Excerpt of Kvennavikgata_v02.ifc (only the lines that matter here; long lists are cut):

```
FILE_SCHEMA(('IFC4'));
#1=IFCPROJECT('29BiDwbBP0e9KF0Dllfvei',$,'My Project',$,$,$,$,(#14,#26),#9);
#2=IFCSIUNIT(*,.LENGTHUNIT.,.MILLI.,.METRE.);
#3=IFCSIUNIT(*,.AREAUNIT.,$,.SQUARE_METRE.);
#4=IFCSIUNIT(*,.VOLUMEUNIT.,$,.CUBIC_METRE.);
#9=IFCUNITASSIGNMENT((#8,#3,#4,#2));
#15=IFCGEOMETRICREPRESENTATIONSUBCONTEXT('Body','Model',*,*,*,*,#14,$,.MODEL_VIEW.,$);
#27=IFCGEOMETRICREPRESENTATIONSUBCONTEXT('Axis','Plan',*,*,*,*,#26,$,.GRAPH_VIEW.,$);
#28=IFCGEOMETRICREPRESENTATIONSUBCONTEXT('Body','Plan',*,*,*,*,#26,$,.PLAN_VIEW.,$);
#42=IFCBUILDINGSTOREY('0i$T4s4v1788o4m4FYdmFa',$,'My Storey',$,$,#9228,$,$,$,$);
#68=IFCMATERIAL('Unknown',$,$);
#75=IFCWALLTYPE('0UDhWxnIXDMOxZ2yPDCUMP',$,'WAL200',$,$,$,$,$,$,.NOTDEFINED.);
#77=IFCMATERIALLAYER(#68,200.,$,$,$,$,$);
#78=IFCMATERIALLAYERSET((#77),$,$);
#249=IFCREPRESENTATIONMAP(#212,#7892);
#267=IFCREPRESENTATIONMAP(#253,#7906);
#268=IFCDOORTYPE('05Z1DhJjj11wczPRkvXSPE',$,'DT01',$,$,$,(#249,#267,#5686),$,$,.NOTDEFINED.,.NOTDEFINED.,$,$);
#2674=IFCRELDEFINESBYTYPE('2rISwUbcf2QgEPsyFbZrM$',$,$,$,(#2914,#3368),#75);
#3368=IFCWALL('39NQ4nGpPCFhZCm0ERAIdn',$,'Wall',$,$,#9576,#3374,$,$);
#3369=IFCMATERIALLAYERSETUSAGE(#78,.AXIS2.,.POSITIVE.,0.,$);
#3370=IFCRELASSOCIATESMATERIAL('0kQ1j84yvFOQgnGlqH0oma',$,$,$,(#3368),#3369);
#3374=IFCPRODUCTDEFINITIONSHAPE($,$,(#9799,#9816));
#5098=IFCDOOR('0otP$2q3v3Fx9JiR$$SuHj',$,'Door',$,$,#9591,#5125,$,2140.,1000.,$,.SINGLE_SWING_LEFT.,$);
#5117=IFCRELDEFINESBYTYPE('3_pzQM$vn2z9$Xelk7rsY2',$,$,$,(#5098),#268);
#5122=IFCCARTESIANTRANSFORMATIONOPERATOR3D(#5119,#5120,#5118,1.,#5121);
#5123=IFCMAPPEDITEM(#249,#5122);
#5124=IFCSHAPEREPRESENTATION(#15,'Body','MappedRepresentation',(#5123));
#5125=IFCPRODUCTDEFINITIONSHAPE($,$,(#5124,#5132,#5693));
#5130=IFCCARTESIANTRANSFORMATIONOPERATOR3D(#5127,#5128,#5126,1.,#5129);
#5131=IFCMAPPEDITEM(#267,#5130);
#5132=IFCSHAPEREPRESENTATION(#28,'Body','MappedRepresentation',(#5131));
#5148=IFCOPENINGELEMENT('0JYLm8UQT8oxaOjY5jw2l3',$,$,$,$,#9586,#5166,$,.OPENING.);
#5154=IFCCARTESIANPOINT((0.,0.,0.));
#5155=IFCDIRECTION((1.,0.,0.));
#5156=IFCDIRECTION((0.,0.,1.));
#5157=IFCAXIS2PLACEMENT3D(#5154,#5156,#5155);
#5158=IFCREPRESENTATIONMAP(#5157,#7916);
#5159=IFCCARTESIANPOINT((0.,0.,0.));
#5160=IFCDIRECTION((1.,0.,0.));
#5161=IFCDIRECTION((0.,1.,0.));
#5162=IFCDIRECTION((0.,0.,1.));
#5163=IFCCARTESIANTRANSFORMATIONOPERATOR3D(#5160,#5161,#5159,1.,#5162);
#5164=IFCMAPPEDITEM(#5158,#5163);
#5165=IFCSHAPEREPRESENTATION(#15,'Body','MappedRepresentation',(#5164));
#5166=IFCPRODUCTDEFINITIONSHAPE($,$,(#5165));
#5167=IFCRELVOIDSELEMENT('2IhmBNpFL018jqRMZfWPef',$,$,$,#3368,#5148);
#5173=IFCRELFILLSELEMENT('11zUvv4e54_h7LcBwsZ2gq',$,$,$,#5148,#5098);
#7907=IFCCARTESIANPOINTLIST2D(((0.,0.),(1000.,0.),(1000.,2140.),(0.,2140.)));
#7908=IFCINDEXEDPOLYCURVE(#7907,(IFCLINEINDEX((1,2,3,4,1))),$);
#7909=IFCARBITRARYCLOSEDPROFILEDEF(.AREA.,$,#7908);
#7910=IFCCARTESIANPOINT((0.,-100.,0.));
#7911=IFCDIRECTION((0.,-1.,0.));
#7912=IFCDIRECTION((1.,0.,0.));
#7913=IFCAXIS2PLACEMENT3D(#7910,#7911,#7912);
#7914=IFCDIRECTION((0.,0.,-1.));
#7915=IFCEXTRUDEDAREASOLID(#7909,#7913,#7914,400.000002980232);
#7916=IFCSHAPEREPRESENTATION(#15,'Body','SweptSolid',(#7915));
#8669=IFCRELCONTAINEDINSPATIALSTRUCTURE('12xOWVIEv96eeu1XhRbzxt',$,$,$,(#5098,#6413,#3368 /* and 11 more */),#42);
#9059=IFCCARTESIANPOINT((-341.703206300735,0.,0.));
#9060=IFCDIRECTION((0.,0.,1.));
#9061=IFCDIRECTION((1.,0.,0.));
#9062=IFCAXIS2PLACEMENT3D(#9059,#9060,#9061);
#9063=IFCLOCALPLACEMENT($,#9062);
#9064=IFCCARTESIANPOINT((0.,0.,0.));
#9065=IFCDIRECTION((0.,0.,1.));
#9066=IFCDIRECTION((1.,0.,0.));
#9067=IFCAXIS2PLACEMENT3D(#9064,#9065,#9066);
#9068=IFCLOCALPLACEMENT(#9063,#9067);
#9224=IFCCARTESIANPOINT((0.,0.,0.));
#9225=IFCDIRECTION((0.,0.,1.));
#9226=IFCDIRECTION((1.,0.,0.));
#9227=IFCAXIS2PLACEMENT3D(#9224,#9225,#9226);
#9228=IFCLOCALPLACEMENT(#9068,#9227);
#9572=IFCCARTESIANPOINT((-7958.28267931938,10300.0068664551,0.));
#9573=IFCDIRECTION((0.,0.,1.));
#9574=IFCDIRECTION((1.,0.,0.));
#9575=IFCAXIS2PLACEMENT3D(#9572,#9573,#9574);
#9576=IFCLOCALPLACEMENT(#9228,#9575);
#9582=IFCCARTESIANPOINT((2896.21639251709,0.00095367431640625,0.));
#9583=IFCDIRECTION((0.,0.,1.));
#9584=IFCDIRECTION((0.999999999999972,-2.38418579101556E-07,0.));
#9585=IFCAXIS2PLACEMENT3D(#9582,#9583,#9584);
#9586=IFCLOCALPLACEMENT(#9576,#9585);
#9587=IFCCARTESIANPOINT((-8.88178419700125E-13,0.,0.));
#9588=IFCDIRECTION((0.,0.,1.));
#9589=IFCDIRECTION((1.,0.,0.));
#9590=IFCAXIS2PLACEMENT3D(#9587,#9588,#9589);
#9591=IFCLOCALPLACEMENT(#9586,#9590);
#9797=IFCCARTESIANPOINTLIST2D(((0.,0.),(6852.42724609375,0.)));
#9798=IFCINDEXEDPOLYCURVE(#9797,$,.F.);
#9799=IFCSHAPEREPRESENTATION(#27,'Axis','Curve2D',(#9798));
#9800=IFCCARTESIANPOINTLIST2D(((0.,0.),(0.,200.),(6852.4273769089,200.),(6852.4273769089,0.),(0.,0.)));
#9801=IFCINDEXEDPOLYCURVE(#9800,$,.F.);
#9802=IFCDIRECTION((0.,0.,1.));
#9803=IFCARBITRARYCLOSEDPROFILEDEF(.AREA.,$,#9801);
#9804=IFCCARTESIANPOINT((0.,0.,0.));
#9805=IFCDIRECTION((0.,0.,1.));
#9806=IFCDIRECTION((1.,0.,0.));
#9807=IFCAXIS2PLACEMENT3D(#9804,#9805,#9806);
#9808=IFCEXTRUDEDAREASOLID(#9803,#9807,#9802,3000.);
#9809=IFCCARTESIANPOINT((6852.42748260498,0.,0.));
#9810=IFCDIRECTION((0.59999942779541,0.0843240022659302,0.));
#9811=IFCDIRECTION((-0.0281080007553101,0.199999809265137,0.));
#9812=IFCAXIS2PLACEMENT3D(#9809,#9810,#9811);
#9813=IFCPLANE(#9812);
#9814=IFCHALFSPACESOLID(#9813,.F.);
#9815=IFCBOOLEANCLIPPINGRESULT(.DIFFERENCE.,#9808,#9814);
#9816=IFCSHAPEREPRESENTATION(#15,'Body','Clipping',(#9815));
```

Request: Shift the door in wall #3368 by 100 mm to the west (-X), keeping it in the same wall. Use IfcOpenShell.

```python
import ifcopenshell
import ifcopenshell.api.geometry
import ifcopenshell.util.placement

model = ifcopenshell.open("Kvennavikgata_v02.ifc")

door = model.by_id(5098)
opening = door.FillsVoids[0].RelatingOpeningElement
wall = opening.VoidsElements[0].RelatingBuildingElement

wall_matrix = ifcopenshell.util.placement.get_local_placement(wall.ObjectPlacement)
shift = wall_matrix[:3, 0] * -100.0
before = ifcopenshell.util.placement.get_local_placement(door.ObjectPlacement)[:3, 3].copy()

# The door is placed relative to its opening, so it follows when the opening moves.
matrix = ifcopenshell.util.placement.get_local_placement(opening.ObjectPlacement)
matrix[:3, 3] += shift
ifcopenshell.api.geometry.edit_object_placement(
    model, product=opening, matrix=matrix, is_si=False, should_transform_children=True
)

after = ifcopenshell.util.placement.get_local_placement(door.ObjectPlacement)[:3, 3]
print("door moved by", (after - before).round(3) + 0.0)

model.write("Kvennavikgata_v02_v2.ifc")
```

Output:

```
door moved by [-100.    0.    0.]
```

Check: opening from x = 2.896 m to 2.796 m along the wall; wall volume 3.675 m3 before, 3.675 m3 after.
